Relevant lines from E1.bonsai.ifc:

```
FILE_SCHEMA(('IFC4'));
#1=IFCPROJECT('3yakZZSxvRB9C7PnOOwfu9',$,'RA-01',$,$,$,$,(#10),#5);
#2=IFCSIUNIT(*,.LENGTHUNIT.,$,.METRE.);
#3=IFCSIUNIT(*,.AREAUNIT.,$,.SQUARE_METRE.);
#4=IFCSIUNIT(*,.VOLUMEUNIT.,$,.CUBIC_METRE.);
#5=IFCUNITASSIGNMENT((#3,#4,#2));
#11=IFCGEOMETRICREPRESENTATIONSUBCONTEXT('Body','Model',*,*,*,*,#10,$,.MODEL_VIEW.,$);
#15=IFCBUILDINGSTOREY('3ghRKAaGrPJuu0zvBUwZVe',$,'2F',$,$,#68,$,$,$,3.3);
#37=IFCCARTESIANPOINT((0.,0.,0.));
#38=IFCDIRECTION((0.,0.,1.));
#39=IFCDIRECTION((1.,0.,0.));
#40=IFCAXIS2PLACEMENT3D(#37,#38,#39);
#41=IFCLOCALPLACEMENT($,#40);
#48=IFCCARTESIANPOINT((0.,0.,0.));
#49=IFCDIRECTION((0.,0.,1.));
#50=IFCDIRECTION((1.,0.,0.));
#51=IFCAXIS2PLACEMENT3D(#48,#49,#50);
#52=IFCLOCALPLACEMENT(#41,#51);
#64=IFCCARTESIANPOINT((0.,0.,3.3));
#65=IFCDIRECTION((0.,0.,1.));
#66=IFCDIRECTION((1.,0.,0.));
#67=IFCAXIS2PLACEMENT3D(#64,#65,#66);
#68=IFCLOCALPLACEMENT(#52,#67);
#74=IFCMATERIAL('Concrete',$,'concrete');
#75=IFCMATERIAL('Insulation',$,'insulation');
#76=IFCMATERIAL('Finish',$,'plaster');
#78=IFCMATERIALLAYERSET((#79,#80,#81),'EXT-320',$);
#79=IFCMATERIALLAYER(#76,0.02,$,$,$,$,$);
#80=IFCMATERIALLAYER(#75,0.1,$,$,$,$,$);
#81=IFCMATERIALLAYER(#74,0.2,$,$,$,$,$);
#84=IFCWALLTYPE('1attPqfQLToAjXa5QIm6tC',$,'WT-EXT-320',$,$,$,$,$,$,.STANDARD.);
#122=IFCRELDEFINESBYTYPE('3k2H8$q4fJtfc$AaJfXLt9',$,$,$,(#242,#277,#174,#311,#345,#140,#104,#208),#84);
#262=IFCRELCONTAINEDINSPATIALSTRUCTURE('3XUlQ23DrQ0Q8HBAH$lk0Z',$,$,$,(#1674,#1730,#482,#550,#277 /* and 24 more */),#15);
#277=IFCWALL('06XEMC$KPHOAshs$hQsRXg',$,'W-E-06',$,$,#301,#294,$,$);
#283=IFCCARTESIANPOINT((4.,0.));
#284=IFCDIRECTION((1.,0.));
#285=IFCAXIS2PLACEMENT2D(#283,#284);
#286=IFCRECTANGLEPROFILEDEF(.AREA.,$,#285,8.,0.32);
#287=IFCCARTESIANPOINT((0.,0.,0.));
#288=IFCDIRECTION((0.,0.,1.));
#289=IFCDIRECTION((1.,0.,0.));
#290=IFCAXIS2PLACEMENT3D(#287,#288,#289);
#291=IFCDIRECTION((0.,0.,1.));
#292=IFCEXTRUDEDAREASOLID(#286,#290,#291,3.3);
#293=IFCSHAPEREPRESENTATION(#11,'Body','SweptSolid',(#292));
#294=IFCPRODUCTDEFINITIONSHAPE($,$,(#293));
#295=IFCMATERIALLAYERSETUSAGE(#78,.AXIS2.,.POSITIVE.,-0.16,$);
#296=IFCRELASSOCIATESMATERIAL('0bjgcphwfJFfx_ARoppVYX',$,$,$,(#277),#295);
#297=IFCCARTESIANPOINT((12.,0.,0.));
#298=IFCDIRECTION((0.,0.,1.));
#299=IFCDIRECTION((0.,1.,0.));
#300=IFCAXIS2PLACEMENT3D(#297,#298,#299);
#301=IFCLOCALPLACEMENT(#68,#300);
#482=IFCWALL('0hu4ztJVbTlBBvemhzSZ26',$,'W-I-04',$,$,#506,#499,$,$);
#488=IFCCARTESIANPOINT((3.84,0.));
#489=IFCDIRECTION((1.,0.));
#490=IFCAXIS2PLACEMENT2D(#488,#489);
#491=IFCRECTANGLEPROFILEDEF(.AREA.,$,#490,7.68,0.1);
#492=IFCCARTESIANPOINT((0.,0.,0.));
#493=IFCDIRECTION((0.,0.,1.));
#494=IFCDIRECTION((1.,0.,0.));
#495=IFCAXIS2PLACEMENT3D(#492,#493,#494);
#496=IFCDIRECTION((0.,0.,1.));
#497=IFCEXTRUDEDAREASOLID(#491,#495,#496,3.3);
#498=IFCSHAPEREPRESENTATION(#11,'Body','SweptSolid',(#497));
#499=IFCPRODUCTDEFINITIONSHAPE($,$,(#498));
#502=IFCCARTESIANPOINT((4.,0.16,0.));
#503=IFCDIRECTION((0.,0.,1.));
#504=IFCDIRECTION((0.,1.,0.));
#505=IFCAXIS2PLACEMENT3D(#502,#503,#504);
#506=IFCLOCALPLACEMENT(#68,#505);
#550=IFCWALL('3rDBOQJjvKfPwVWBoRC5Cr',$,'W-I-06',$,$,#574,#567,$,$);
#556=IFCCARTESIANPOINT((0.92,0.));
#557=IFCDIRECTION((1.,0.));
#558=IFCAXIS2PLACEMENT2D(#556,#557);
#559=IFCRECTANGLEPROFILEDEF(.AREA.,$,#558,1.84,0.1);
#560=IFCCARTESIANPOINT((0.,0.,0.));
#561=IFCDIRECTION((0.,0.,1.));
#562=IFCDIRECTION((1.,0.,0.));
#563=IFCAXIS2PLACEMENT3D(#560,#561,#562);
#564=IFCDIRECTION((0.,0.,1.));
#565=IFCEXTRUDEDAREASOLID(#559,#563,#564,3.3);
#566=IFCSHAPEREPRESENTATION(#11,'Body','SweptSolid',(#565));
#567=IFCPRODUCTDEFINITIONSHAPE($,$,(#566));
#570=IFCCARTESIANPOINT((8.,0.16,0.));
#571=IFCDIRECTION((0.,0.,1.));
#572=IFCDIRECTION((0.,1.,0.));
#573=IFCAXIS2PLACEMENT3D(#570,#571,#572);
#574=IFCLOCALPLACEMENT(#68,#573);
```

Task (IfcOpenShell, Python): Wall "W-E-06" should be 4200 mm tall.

```python
import ifcopenshell
import ifcopenshell.geom
import ifcopenshell.util.representation
import ifcopenshell.util.shape

model = ifcopenshell.open("E1.bonsai.ifc")
settings = ifcopenshell.geom.settings()


def volume(element):
    """Net volume in cubic metres, openings subtracted."""
    shape = ifcopenshell.geom.create_shape(settings, element)
    return ifcopenshell.util.shape.get_volume(shape.geometry)


wall = model.by_guid("06XEMC$KPHOAshs$hQsRXg")
before = volume(wall)

body = ifcopenshell.util.representation.get_representation(wall, "Model", "Body")
solid = body.Items[0]
old_height = solid.Depth
solid.Depth = 4.2
after = volume(wall)

print(f"height {old_height:g} -> {solid.Depth:g}, volume {before:.3f} -> {after:.3f} m3")

model.write("E1.bonsai-out.ifc")
```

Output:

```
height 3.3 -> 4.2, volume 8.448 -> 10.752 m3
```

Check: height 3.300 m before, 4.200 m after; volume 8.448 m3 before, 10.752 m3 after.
